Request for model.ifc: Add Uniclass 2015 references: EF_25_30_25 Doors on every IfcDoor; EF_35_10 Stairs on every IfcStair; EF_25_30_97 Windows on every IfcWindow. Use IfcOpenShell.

First a look at what the model holds.

```python
import ifcopenshell

model = ifcopenshell.open("model.ifc")
print(model.schema)
print("classifications:", [c.Name for c in model.by_type("IfcClassification")])
for ifc_class in ("IfcDoor", "IfcRoof", "IfcStair", "IfcWall", "IfcWindow"):
    print(ifc_class, len(model.by_type(ifc_class)))
```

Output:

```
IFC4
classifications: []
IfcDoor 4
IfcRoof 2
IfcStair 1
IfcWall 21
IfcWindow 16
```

```python
import ifcopenshell
import ifcopenshell.api.classification

model = ifcopenshell.open("model.ifc")

system = ifcopenshell.api.classification.add_classification(model, classification="Uniclass 2015")

codes = {
    "IfcDoor": ("EF_25_30_25", "Doors"),
    "IfcStair": ("EF_35_10", "Stairs"),
    "IfcWindow": ("EF_25_30_97", "Windows"),
}
for ifc_class, (code, name) in codes.items():
    products = model.by_type(ifc_class)
    ifcopenshell.api.classification.add_reference(
        model, products=products, classification=system, identification=code, name=name
    )
    print(code, len(products))

model.write("model_rev.ifc")
```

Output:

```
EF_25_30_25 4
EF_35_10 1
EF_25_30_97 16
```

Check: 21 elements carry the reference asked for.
